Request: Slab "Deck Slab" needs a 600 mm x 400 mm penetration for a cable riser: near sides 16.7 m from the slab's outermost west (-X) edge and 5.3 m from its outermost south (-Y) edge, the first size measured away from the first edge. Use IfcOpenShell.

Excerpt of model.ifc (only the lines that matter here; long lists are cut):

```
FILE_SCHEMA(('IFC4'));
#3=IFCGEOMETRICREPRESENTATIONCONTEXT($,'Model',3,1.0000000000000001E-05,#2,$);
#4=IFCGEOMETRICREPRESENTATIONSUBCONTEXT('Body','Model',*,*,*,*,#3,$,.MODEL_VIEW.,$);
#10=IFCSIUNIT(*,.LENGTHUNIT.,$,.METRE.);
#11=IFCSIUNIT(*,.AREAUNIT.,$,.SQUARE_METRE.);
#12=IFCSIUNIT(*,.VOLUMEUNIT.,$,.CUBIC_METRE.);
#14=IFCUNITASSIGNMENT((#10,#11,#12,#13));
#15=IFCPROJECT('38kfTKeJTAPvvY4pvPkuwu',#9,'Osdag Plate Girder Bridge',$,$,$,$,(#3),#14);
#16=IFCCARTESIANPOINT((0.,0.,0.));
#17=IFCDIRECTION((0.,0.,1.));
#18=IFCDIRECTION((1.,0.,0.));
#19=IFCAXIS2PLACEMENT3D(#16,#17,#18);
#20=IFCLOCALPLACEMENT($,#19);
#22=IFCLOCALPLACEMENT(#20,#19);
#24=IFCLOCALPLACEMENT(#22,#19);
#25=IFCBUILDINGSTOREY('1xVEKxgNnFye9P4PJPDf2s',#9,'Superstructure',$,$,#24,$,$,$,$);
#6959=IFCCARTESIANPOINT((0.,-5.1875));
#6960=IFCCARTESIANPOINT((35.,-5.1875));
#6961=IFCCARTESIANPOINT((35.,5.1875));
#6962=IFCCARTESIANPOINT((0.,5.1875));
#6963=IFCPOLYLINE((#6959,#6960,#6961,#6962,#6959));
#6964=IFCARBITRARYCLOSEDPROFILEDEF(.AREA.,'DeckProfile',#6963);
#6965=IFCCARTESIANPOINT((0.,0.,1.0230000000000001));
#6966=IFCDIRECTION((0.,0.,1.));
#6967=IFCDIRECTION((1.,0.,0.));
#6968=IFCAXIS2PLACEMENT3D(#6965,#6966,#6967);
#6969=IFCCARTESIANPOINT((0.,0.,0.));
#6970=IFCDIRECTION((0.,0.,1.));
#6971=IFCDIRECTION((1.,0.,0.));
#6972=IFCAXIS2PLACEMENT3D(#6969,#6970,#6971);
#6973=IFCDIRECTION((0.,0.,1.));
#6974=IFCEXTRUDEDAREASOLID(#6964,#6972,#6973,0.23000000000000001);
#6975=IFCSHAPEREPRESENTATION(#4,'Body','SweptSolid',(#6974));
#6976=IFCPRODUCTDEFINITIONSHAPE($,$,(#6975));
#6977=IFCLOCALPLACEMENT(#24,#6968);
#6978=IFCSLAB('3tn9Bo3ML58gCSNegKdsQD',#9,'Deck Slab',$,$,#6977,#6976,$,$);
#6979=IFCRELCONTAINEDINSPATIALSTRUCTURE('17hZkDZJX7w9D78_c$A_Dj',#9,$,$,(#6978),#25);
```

```python
import numpy as np
import ifcopenshell
import ifcopenshell.api.feature
import ifcopenshell.api.geometry
import ifcopenshell.api.root
import ifcopenshell.geom
import ifcopenshell.util.placement
import ifcopenshell.util.representation
import ifcopenshell.util.shape
import ifcopenshell.util.unit

model = ifcopenshell.open("model.ifc")
unit_scale = ifcopenshell.util.unit.calculate_unit_scale(model)
settings = ifcopenshell.geom.settings()


def volume(element):
    """Net volume in cubic metres, openings subtracted."""
    shape = ifcopenshell.geom.create_shape(settings, element)
    return ifcopenshell.util.shape.get_volume(shape.geometry)


slab = model.by_guid("3tn9Bo3ML58gCSNegKdsQD")
before = volume(slab)

# Extent in the slab's own axes, in metres. The edges named are its -X and -Y sides.
slab_shape = ifcopenshell.geom.create_shape(settings, slab)
vertices = ifcopenshell.util.shape.get_vertices(slab_shape.geometry)
x_min, y_min, bottom = vertices.min(axis=0)
top = vertices[:, 2].max()

opening = ifcopenshell.api.root.create_entity(model, ifc_class="IfcOpeningElement", name="Cable riser opening", predefined_type="OPENING")
context = ifcopenshell.util.representation.get_context(model, "Model", "Body", "MODEL_VIEW")
width, depth = 0.6, 0.4
outline = [(0.0, 0.0), (width, 0.0), (width, depth), (0.0, depth), (0.0, 0.0)]
# Overshoot both faces by 50 mm so the cut is clean.
shape = ifcopenshell.api.geometry.add_slab_representation(
    model, context=context, depth=top - bottom + 0.1, polyline=outline
)
ifcopenshell.api.geometry.assign_representation(model, product=opening, representation=shape)

matrix = ifcopenshell.util.placement.get_local_placement(slab.ObjectPlacement)
matrix[:, 3] = matrix @ np.append(np.array([x_min + 16.7, y_min + 5.3, bottom - 0.05]) / unit_scale, 1.0)
ifcopenshell.api.geometry.edit_object_placement(model, product=opening, matrix=matrix, is_si=False)
ifcopenshell.api.feature.add_feature(model, feature=opening, element=slab)

after = volume(slab)

print(f"slab volume {before:.3f} -> {after:.3f} m3")

model.write("model_rev.ifc")
```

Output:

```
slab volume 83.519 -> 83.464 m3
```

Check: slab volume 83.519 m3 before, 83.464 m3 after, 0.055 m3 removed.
